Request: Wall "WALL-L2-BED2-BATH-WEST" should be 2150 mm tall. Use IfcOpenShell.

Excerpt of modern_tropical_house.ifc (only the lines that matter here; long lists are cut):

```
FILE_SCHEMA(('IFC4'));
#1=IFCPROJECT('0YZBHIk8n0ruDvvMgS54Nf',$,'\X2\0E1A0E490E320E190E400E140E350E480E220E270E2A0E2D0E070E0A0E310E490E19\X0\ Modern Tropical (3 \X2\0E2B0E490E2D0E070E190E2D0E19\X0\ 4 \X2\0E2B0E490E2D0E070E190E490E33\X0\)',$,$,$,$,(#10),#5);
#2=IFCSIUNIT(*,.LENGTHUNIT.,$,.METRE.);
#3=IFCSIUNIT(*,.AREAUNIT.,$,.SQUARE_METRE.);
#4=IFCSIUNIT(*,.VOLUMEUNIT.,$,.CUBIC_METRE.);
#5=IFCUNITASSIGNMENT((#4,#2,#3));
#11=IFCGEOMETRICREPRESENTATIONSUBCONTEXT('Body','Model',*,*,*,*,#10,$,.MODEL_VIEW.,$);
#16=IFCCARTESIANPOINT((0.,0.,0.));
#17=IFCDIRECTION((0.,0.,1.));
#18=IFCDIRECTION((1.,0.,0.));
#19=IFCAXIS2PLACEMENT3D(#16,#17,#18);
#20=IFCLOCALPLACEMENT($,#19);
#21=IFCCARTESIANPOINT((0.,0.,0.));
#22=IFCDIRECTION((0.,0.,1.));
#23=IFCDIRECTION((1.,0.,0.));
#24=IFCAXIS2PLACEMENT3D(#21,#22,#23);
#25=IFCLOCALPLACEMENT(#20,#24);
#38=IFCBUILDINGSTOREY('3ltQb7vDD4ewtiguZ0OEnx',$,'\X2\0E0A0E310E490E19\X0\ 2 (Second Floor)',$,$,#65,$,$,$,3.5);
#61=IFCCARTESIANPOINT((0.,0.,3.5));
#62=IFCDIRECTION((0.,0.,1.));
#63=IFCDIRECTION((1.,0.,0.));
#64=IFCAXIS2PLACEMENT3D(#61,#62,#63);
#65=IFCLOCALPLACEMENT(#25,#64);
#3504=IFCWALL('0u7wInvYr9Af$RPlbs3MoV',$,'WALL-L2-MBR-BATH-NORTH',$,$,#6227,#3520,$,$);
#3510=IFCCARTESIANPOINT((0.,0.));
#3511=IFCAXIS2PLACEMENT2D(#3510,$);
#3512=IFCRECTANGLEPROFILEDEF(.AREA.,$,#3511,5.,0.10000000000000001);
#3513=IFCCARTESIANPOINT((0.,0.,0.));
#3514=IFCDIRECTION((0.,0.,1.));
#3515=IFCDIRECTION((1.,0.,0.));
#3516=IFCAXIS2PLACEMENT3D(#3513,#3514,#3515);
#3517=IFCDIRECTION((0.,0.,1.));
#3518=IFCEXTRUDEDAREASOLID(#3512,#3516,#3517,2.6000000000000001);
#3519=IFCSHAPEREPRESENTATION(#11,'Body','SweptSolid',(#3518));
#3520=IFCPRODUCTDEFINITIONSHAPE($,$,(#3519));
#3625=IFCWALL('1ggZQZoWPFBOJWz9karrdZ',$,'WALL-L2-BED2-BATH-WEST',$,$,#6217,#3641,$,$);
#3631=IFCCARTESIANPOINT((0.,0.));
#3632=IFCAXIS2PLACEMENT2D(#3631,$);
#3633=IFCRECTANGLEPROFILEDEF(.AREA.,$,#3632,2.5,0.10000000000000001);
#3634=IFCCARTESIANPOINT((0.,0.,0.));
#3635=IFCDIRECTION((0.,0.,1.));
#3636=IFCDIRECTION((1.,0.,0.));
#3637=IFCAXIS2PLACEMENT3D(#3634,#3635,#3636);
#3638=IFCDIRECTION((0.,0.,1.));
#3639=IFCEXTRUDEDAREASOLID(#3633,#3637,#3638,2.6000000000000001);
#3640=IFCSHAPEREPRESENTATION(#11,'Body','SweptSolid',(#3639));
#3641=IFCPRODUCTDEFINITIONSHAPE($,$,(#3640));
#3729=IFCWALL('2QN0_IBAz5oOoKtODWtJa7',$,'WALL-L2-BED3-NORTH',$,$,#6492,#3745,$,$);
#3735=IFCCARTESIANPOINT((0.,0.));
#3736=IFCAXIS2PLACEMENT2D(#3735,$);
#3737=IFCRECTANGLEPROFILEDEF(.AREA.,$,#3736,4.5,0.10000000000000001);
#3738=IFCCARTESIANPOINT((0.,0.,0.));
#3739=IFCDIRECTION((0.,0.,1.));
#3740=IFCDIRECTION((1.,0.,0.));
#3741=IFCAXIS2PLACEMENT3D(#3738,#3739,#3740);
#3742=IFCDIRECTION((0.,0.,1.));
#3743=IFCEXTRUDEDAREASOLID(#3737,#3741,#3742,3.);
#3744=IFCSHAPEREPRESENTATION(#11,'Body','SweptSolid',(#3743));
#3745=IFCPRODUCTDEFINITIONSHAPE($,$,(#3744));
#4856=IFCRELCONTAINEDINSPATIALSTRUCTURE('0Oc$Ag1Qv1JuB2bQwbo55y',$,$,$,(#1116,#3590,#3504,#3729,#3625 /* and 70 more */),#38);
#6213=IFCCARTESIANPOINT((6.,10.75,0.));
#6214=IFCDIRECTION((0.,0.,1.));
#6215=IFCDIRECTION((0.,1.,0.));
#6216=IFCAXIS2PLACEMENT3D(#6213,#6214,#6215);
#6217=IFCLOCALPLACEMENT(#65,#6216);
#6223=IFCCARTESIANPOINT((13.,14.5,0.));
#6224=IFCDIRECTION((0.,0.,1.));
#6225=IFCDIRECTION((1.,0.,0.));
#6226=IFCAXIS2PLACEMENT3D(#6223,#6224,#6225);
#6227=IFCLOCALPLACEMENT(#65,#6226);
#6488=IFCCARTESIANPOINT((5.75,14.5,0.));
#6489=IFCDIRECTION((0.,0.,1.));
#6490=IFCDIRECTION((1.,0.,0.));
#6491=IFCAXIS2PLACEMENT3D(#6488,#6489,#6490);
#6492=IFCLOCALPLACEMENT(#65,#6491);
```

```python
import ifcopenshell
import ifcopenshell.geom
import ifcopenshell.util.representation
import ifcopenshell.util.shape
import ifcopenshell.util.unit

model = ifcopenshell.open("modern_tropical_house.ifc")
unit_scale = ifcopenshell.util.unit.calculate_unit_scale(model)
settings = ifcopenshell.geom.settings()


def volume(element):
    """Net volume in cubic metres, openings subtracted."""
    shape = ifcopenshell.geom.create_shape(settings, element)
    return ifcopenshell.util.shape.get_volume(shape.geometry)


wall = model.by_id(3625)
before = volume(wall)

body = ifcopenshell.util.representation.get_representation(wall, "Model", "Body")
solid = body.Items[0]
old_height = solid.Depth
solid.Depth = 2.15 / unit_scale
after = volume(wall)

print(f"height {old_height:g} -> {solid.Depth:g}, volume {before:.3f} -> {after:.3f} m3")

model.write("modern_tropical_house_rev.ifc")
```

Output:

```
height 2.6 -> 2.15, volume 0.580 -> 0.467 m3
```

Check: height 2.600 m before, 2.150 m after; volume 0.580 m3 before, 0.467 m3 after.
